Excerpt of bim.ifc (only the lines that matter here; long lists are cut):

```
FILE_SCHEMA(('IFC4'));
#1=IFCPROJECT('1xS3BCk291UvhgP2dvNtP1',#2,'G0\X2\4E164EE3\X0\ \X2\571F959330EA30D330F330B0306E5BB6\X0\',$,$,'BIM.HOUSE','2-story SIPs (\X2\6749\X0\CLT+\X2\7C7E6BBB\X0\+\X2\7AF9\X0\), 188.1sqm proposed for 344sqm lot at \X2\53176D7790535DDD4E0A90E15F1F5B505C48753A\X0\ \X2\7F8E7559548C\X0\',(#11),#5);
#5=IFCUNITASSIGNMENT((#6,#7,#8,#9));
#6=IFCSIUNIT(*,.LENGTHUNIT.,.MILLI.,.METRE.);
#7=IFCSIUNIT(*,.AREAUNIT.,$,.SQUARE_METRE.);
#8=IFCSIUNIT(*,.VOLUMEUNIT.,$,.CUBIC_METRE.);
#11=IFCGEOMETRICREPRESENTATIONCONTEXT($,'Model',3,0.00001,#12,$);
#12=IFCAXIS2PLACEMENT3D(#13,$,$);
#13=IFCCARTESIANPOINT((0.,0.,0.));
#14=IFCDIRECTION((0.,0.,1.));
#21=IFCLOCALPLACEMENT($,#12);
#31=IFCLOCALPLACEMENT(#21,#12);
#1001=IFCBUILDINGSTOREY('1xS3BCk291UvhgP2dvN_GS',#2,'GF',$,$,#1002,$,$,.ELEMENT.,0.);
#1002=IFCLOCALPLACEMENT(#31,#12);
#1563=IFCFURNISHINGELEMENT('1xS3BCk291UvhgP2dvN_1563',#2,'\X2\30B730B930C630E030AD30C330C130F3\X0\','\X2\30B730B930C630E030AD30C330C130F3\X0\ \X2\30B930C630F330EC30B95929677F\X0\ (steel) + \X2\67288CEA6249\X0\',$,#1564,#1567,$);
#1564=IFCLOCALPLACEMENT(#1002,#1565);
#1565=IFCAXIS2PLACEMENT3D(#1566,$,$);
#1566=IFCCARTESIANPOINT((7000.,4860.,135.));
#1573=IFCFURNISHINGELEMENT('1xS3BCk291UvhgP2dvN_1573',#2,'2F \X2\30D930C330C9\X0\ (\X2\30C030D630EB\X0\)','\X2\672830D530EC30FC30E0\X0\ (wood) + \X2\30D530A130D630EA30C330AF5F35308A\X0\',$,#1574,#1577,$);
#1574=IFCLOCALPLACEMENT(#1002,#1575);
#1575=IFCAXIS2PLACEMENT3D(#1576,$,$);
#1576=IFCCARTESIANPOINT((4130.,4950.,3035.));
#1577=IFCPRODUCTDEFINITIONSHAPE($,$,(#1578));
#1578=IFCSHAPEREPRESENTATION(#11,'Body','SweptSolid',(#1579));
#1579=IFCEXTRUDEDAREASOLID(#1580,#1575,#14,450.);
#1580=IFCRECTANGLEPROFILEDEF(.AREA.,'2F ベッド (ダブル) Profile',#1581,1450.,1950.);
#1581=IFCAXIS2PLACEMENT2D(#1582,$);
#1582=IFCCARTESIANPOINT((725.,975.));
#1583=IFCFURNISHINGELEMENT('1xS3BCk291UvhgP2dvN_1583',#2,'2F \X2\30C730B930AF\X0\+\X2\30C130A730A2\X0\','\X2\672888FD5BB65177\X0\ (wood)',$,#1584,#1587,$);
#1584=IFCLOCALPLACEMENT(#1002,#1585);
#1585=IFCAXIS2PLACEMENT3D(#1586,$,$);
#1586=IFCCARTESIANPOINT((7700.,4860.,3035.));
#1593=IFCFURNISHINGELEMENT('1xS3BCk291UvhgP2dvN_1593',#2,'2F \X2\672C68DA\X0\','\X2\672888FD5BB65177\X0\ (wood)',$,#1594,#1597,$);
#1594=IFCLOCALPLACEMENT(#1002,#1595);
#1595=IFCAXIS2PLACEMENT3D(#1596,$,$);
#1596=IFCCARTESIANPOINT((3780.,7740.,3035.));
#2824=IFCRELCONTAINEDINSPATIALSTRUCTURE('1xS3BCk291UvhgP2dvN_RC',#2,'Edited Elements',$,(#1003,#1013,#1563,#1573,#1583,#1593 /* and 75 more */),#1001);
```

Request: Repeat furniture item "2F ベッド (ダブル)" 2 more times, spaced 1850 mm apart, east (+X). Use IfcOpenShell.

```python
import numpy as np
import ifcopenshell
import ifcopenshell.api.geometry
import ifcopenshell.api.root
import ifcopenshell.util.element
import ifcopenshell.util.placement

model = ifcopenshell.open("bim.ifc")


def reuse_history(source, copy):
    """copy_class also copies each property set's owner history, people and application; keep the originals."""
    for rel in copy.IsDefinedBy:
        if rel.is_a("IfcRelDefinesByProperties") and (history := rel.RelatingPropertyDefinition.OwnerHistory):
            rel.RelatingPropertyDefinition.OwnerHistory = source.OwnerHistory
            ifcopenshell.util.element.remove_deep2(model, history)


source = model.by_id(1573)
base = ifcopenshell.util.placement.get_local_placement(source.ObjectPlacement)
step = np.array([1.0, 0.0, 0.0]) * 1850.0

for i in range(1, 3):
    copy = ifcopenshell.api.root.copy_class(model, product=source)
    copy.Representation = ifcopenshell.util.element.copy_deep(
        model, source.Representation, exclude=["IfcGeometricRepresentationContext", "IfcRepresentationMap"]
    )
    reuse_history(source, copy)
    matrix = base.copy()
    matrix[:3, 3] += i * step
    print("added at", matrix[:3, 3].round(3) + 0.0)
    ifcopenshell.api.geometry.edit_object_placement(model, product=copy, matrix=matrix, is_si=False)

model.write("bim_rev.ifc")
```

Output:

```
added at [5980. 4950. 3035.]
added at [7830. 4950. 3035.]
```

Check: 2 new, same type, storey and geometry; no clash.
